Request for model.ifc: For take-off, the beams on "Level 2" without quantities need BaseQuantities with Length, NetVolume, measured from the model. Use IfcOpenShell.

First a look at what the model holds.

```python
import ifcopenshell
import ifcopenshell.util.element
import ifcopenshell.util.unit

model = ifcopenshell.open("model.ifc")
print(model.schema)
for unit_type in ("LENGTHUNIT", "AREAUNIT", "VOLUMEUNIT"):
    print(unit_type, ifcopenshell.util.unit.calculate_unit_scale(model, unit_type))
storey = next(s for s in model.by_type("IfcBuildingStorey") if s.Name == "Level 2")
beams = [e for e in ifcopenshell.util.element.get_decomposition(storey) if e.is_a("IfcBeam")]
for e in sorted(beams, key=lambda e: e.id()):
    print(e.id(), e.is_a(), e.Name, list(ifcopenshell.util.element.get_psets(e, qtos_only=True)), sep=" | ")
```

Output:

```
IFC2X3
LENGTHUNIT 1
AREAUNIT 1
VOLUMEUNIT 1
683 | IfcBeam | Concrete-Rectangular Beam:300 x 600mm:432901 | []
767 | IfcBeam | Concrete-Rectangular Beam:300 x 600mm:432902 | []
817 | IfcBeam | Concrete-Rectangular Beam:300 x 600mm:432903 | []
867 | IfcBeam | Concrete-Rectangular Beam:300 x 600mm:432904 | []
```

```python
import ifcopenshell
import ifcopenshell.api.pset
import ifcopenshell.geom
import ifcopenshell.util.element
import ifcopenshell.util.shape
import ifcopenshell.util.unit

model = ifcopenshell.open("model.ifc")
unit_scale = ifcopenshell.util.unit.calculate_unit_scale(model)
volume_scale = ifcopenshell.util.unit.calculate_unit_scale(model, "VOLUMEUNIT")
settings = ifcopenshell.geom.settings()

storey = next(s for s in model.by_type("IfcBuildingStorey") if s.Name == "Level 2")
beams = [e for e in ifcopenshell.util.element.get_decomposition(storey) if e.is_a("IfcBeam")]

for e in sorted(beams, key=lambda e: e.id()):
    if ifcopenshell.util.element.get_psets(e, qtos_only=True, should_inherit=False):
        continue
    # Geometry comes back in metres, in the element's own axes.
    shape = ifcopenshell.geom.create_shape(settings, e)
    values = {
        "Length": ifcopenshell.util.shape.get_max_xyz(shape.geometry) / unit_scale,
        "NetVolume": ifcopenshell.util.shape.get_volume(shape.geometry) / volume_scale,
    }
    qto = ifcopenshell.api.pset.add_qto(model, product=e, name="BaseQuantities")
    ifcopenshell.api.pset.edit_qto(model, qto=qto, properties=values)
    print(e.id(), {k: round(v, 3) for k, v in values.items()})

model.write("model_v2.ifc")
```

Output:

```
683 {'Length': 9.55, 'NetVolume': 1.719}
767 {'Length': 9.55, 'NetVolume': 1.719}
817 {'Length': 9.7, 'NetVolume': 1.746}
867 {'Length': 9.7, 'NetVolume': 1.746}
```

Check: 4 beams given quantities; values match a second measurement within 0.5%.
